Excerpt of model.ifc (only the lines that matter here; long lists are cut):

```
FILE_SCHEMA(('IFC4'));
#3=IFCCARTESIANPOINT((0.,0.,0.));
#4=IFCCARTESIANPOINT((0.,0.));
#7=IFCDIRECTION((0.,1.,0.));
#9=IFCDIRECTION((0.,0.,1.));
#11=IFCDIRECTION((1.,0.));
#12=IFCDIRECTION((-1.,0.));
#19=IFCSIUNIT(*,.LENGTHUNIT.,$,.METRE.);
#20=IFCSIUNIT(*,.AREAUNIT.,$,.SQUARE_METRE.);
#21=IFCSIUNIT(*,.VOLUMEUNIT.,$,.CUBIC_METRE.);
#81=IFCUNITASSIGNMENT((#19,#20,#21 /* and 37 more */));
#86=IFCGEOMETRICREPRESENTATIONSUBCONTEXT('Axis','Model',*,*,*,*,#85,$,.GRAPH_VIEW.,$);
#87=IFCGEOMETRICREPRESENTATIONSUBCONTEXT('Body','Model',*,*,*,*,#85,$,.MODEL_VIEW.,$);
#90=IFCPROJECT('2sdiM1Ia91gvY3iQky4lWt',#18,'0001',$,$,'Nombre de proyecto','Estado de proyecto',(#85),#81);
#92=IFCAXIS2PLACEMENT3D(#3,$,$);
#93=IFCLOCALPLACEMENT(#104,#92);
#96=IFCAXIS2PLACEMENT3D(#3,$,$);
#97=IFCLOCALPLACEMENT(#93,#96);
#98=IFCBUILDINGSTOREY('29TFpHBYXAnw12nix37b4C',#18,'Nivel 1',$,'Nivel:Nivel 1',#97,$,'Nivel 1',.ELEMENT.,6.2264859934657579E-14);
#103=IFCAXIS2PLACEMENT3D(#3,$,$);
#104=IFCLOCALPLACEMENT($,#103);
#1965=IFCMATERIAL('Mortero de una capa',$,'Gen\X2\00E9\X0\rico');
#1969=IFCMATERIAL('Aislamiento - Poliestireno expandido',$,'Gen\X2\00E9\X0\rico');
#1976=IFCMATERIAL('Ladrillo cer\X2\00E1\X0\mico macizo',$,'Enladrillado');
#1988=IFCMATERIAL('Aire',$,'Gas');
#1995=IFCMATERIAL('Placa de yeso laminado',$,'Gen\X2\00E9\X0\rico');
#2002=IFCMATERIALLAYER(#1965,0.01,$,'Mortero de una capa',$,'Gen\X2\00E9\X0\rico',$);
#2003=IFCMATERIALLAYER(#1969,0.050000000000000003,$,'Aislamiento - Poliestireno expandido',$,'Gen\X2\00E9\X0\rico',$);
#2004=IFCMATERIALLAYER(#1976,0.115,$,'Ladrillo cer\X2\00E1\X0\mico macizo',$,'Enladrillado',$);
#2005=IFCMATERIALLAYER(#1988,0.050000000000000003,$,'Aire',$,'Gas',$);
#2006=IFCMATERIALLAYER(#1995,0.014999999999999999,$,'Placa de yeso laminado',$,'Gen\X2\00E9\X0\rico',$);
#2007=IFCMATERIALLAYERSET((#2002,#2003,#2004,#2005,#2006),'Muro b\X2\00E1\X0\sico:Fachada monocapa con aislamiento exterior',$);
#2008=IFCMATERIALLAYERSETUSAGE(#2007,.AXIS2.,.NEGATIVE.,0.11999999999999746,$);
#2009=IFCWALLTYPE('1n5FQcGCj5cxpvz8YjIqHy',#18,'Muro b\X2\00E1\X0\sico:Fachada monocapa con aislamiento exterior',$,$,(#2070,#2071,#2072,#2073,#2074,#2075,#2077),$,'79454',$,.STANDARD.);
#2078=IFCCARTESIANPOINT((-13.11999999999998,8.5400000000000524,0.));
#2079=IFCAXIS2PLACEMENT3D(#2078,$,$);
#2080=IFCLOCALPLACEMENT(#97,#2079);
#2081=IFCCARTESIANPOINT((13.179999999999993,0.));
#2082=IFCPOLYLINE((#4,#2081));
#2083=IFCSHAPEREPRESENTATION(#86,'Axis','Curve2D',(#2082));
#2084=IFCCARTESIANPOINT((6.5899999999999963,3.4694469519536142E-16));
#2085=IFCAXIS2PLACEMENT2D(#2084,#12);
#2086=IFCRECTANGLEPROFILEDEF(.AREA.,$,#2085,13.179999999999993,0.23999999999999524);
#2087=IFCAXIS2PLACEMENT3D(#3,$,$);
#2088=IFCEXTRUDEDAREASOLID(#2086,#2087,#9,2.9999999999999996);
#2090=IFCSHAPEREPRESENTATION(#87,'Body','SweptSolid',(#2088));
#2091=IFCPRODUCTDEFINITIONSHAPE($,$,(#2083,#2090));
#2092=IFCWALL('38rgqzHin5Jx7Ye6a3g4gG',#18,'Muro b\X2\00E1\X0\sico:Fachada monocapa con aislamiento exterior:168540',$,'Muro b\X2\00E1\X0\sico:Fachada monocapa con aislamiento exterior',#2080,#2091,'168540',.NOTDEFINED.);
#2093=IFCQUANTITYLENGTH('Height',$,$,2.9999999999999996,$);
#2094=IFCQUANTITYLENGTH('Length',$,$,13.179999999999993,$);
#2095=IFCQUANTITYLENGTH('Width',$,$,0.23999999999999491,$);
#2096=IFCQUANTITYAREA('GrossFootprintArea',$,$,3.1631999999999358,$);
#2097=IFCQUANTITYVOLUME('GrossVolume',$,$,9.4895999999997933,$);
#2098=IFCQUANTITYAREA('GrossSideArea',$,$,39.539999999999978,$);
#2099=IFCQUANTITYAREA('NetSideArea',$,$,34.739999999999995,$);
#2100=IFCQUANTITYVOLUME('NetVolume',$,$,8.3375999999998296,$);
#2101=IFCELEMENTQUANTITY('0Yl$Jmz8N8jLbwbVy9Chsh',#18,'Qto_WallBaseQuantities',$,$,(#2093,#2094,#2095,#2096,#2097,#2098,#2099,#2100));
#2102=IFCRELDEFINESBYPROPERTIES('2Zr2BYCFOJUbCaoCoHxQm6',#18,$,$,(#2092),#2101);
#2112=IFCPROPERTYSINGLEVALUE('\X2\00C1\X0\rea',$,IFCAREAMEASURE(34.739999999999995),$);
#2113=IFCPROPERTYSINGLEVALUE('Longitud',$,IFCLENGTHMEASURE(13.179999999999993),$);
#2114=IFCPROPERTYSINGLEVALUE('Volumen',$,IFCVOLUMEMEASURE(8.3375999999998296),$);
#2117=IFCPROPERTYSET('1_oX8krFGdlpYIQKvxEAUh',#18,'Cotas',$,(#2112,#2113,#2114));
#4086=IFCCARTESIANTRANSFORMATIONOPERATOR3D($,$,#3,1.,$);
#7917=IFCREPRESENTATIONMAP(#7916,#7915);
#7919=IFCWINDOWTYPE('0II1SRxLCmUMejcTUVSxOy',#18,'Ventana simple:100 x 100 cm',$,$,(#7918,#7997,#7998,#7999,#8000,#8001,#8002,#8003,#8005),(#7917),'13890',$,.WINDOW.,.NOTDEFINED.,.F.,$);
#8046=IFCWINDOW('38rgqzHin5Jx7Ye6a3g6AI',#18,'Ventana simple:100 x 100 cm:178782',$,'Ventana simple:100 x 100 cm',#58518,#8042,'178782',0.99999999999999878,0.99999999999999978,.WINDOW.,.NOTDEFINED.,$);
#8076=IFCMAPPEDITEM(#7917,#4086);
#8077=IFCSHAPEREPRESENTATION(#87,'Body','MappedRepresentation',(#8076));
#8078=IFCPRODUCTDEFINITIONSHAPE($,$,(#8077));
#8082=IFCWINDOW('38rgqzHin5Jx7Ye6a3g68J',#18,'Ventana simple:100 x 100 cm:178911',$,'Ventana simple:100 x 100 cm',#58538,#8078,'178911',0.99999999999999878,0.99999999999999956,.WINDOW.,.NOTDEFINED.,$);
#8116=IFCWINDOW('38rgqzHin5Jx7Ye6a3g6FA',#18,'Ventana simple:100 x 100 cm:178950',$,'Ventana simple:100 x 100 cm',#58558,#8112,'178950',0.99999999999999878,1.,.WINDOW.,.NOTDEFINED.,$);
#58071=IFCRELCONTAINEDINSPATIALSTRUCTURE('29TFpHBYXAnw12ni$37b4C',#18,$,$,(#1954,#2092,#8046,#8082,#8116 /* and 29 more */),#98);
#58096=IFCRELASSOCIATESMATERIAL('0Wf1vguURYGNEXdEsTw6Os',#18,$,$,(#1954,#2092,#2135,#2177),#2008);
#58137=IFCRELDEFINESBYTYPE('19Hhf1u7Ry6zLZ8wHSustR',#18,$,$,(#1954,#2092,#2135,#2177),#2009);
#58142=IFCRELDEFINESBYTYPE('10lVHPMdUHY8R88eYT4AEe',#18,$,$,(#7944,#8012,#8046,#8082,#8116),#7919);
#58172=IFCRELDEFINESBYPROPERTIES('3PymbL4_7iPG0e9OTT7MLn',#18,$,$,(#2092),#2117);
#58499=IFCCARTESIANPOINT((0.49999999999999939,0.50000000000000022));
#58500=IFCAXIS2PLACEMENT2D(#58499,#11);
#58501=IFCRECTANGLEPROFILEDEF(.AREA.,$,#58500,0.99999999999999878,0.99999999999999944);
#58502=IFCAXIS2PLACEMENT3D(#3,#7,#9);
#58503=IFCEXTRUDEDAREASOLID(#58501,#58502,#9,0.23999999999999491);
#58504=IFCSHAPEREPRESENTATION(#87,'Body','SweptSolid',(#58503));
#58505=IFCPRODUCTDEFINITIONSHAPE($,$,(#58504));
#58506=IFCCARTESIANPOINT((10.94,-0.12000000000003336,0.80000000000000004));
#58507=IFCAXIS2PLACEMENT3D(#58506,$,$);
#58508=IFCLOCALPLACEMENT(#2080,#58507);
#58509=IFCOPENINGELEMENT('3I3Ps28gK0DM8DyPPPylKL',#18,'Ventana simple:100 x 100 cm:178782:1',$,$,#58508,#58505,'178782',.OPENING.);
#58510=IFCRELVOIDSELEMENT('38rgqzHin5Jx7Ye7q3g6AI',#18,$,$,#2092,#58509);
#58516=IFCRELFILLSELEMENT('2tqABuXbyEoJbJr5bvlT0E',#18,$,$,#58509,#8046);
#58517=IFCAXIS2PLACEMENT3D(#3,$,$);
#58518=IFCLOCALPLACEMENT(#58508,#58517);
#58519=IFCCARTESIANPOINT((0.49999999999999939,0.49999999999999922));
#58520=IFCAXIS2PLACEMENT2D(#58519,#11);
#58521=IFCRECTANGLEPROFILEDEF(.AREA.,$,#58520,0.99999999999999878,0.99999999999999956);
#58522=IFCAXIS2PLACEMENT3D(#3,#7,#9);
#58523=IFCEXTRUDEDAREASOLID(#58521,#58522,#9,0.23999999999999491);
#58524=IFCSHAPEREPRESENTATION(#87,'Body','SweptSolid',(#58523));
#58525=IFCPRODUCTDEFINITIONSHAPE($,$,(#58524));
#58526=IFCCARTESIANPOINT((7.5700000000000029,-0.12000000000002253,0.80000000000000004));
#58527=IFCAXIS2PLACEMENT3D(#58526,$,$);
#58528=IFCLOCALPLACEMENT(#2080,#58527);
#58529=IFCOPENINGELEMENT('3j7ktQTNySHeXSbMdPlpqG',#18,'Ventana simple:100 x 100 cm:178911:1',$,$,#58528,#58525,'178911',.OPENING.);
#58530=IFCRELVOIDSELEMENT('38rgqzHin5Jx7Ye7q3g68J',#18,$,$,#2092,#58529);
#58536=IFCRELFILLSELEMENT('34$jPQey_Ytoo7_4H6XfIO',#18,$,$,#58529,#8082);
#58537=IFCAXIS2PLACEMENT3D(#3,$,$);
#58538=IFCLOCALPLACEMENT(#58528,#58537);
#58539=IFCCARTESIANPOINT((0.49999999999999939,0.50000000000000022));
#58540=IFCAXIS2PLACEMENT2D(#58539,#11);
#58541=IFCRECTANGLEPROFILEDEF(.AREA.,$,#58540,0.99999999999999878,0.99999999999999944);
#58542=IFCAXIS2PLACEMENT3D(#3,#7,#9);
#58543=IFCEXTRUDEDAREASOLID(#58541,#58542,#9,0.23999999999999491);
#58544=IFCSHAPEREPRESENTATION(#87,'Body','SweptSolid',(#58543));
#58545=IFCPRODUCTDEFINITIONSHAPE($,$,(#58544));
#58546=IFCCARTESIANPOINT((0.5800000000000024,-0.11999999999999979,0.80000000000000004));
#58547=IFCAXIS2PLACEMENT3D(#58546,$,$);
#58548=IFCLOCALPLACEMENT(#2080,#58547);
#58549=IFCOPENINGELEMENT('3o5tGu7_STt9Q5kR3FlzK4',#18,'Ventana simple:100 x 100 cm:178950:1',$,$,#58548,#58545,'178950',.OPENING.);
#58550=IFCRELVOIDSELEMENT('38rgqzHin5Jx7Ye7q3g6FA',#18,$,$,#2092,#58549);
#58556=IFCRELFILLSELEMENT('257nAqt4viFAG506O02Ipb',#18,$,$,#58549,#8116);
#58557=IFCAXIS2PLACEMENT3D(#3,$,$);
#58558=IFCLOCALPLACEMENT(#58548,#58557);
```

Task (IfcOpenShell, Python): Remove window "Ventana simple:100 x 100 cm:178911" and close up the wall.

```python
import ifcopenshell
import ifcopenshell.api.feature
import ifcopenshell.api.pset
import ifcopenshell.api.root
import ifcopenshell.geom
import ifcopenshell.util.element
import ifcopenshell.util.shape
import ifcopenshell.util.unit

model = ifcopenshell.open("model.ifc")
area_scale = ifcopenshell.util.unit.calculate_unit_scale(model, "AREAUNIT")
volume_scale = ifcopenshell.util.unit.calculate_unit_scale(model, "VOLUMEUNIT")
settings = ifcopenshell.geom.settings()


def volume(element):
    """Net volume in cubic metres, openings subtracted."""
    shape = ifcopenshell.geom.create_shape(settings, element)
    return ifcopenshell.util.shape.get_volume(shape.geometry)


window = model.by_guid("38rgqzHin5Jx7Ye6a3g68J")
opening = window.FillsVoids[0].RelatingOpeningElement
wall = opening.VoidsElements[0].RelatingBuildingElement
before = volume(wall)

ifcopenshell.api.root.remove_product(model, product=window)
ifcopenshell.api.feature.remove_feature(model, feature=opening)

after = volume(wall)
thickness = 0.24  # wall thickness in metres

# Update the wall's stored quantities.
qto = model.by_id(ifcopenshell.util.element.get_pset(wall, "Qto_WallBaseQuantities", should_inherit=False)["id"])
ifcopenshell.api.pset.edit_qto(model, qto=qto, properties={
    "NetSideArea": after / thickness / area_scale,
    "NetVolume": after / volume_scale,
})
pset = model.by_id(ifcopenshell.util.element.get_pset(wall, "Cotas", should_inherit=False)["id"])
ifcopenshell.api.pset.edit_pset(model, pset=pset, properties={
    "Área": model.create_entity("IfcAreaMeasure", after / thickness / area_scale),
    "Volumen": model.create_entity("IfcVolumeMeasure", after / volume_scale),
})

print(f"wall volume {before:.3f} -> {after:.3f} m3")

model.write("model_updated.ifc")
```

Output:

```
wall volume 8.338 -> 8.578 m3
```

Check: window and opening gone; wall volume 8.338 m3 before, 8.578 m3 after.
